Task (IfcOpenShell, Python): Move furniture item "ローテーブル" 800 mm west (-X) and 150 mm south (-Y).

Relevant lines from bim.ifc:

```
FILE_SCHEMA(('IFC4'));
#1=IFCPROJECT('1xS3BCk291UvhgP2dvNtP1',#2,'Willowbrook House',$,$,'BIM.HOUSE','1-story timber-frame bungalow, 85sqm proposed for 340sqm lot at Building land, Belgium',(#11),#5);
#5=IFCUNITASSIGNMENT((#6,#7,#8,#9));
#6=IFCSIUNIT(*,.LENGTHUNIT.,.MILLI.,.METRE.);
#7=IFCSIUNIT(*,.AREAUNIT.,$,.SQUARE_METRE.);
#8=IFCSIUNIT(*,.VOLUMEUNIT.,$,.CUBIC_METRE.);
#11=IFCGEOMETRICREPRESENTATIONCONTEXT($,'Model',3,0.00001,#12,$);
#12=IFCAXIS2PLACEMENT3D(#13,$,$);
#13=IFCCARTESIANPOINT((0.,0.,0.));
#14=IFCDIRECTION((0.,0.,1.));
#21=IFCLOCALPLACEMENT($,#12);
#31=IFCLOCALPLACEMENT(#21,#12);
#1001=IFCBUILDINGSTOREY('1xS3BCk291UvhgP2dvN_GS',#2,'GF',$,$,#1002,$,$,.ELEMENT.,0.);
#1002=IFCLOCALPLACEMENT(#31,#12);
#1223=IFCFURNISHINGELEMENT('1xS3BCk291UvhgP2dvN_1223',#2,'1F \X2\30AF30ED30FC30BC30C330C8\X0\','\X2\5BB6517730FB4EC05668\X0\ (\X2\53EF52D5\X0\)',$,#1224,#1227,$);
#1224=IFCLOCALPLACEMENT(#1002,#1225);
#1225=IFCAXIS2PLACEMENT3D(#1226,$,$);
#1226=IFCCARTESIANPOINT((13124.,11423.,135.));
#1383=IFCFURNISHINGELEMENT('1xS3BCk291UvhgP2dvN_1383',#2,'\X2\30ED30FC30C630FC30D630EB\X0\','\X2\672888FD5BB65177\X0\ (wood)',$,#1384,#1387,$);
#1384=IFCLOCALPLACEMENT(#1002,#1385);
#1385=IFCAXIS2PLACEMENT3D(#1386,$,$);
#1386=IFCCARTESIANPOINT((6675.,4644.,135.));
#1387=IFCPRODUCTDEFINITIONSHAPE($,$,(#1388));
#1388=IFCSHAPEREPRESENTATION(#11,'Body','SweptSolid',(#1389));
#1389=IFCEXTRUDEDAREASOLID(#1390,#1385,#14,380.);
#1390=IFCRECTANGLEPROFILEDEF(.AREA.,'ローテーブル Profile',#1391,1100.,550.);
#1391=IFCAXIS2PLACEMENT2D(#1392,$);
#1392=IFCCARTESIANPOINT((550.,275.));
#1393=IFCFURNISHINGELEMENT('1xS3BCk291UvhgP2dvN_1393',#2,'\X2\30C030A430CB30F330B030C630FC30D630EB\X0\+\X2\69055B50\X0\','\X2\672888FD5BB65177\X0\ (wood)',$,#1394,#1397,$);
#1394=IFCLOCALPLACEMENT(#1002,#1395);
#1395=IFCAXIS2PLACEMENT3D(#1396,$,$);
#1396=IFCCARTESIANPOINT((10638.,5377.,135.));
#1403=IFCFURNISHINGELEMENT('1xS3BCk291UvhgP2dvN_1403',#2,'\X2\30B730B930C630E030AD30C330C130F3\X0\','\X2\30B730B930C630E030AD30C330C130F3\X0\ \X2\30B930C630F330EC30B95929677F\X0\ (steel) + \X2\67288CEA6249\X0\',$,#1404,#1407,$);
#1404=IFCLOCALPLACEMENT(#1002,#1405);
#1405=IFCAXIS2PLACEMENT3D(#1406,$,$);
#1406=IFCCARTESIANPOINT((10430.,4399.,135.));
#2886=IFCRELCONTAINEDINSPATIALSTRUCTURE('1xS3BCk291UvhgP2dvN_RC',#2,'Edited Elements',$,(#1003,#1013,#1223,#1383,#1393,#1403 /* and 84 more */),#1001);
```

```python
import ifcopenshell
import ifcopenshell.api.geometry
import ifcopenshell.util.placement
import ifcopenshell.util.unit

model = ifcopenshell.open("bim.ifc")
unit_scale = ifcopenshell.util.unit.calculate_unit_scale(model)

item = model.by_guid("1xS3BCk291UvhgP2dvN_1383")
matrix = ifcopenshell.util.placement.get_local_placement(item.ObjectPlacement)
matrix[0, 3] -= 0.8 / unit_scale
matrix[1, 3] -= 0.15 / unit_scale
ifcopenshell.api.geometry.edit_object_placement(model, product=item, matrix=matrix, is_si=False)

print(ifcopenshell.util.placement.get_local_placement(item.ObjectPlacement).round(3) + 0.0)

model.write("bim-out.ifc")
```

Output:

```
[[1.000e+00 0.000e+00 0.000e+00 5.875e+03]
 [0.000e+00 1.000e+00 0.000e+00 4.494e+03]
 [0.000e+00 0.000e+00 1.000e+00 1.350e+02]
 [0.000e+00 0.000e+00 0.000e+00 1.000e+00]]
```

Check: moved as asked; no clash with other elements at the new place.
